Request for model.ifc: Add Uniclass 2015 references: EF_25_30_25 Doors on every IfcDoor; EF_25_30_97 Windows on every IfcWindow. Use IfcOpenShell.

First a look at what the model holds.

```python
import ifcopenshell

model = ifcopenshell.open("model.ifc")
print(model.schema)
print("classifications:", [c.Name for c in model.by_type("IfcClassification")])
for ifc_class in ("IfcDoor", "IfcRoof", "IfcStair", "IfcWall", "IfcWindow"):
    print(ifc_class, len(model.by_type(ifc_class)))
```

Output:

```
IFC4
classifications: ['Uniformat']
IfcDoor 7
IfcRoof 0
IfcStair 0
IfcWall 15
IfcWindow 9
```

```python
import ifcopenshell
import ifcopenshell.api.classification

model = ifcopenshell.open("model.ifc")

system = ifcopenshell.api.classification.add_classification(model, classification="Uniclass 2015")

codes = {
    "IfcDoor": ("EF_25_30_25", "Doors"),
    "IfcWindow": ("EF_25_30_97", "Windows"),
}
for ifc_class, (code, name) in codes.items():
    products = model.by_type(ifc_class)
    ifcopenshell.api.classification.add_reference(
        model, products=products, classification=system, identification=code, name=name
    )
    print(code, len(products))

model.write("model-out.ifc")
```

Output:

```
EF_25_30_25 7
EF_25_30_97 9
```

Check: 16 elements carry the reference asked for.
